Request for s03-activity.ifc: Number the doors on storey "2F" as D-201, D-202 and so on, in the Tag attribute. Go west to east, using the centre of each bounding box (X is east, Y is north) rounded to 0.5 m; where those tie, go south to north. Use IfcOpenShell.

First a look at what the model holds.

```python
import ifcopenshell
import ifcopenshell.util.element
import ifcopenshell.util.placement

model = ifcopenshell.open("s03-activity.ifc")
print(model.schema)
storey = next(s for s in model.by_type("IfcBuildingStorey") if s.Name == "2F")
doors = [e for e in ifcopenshell.util.element.get_decomposition(storey) if e.is_a("IfcDoor")]
for e in sorted(doors, key=lambda e: e.id()):
    origin = ifcopenshell.util.placement.get_local_placement(e.ObjectPlacement)[:3, 3]
    print(e.id(), e.Tag, e.Name, origin.round(2) + 0.0, sep=" | ")
```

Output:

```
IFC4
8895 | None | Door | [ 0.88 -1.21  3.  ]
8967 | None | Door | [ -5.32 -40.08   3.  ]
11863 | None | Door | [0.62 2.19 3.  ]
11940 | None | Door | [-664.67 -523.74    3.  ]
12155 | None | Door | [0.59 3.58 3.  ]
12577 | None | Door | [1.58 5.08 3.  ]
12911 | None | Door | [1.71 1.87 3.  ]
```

```python
import ifcopenshell
import ifcopenshell.geom
import ifcopenshell.util.element
import ifcopenshell.util.shape

model = ifcopenshell.open("s03-activity.ifc")
settings = ifcopenshell.geom.settings()
settings.set("use-world-coords", True)


def centre(element):
    shape = ifcopenshell.geom.create_shape(settings, element)
    return ifcopenshell.util.shape.get_bbox_centroid(shape.geometry)


storey = next(s for s in model.by_type("IfcBuildingStorey") if s.Name == "2F")
doors = [e for e in ifcopenshell.util.element.get_decomposition(storey) if e.is_a("IfcDoor")]

# Insertion points can sit at a corner or the storey origin, so sort by the geometry (in metres).
centres = {e: centre(e) for e in doors}
doors.sort(key=lambda e: (round(centres[e][0] / 0.5), centres[e][1]))

for i, e in enumerate(doors, start=1):
    number = f"D-2{i:02d}"
    e.Tag = number
    print(e.id(), number)

model.write("s03-activity_rev.ifc")
```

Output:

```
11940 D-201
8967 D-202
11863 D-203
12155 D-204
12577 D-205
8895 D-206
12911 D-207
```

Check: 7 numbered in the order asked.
